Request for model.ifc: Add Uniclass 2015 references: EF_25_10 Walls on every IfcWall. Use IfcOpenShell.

First a look at what the model holds.

```python
import ifcopenshell

model = ifcopenshell.open("model.ifc")
print(model.schema)
print("classifications:", [c.Name for c in model.by_type("IfcClassification")])
for ifc_class in ("IfcDoor", "IfcRoof", "IfcStair", "IfcWall", "IfcWindow"):
    print(ifc_class, len(model.by_type(ifc_class)))
```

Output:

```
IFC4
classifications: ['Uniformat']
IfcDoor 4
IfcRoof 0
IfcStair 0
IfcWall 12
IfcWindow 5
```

```python
import ifcopenshell
import ifcopenshell.api.classification

model = ifcopenshell.open("model.ifc")

system = ifcopenshell.api.classification.add_classification(model, classification="Uniclass 2015")

codes = {
    "IfcWall": ("EF_25_10", "Walls"),
}
for ifc_class, (code, name) in codes.items():
    products = model.by_type(ifc_class)
    ifcopenshell.api.classification.add_reference(
        model, products=products, classification=system, identification=code, name=name
    )
    print(code, len(products))

model.write("model-out.ifc")
```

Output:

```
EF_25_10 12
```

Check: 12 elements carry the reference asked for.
